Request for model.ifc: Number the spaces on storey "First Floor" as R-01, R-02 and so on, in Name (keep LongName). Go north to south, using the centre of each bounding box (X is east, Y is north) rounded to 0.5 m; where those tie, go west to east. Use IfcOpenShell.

First a look at what the model holds.

```python
import ifcopenshell
import ifcopenshell.util.element
import ifcopenshell.util.placement

model = ifcopenshell.open("model.ifc")
print(model.schema)
storey = next(s for s in model.by_type("IfcBuildingStorey") if s.Name == "First Floor")
spaces = [e for e in ifcopenshell.util.element.get_decomposition(storey) if e.is_a("IfcSpace")]
for e in sorted(spaces, key=lambda e: e.id()):
    origin = ifcopenshell.util.placement.get_local_placement(e.ObjectPlacement)[:3, 3]
    print(e.id(), e.Name, e.LongName, origin.round(2) + 0.0, sep=" | ")
```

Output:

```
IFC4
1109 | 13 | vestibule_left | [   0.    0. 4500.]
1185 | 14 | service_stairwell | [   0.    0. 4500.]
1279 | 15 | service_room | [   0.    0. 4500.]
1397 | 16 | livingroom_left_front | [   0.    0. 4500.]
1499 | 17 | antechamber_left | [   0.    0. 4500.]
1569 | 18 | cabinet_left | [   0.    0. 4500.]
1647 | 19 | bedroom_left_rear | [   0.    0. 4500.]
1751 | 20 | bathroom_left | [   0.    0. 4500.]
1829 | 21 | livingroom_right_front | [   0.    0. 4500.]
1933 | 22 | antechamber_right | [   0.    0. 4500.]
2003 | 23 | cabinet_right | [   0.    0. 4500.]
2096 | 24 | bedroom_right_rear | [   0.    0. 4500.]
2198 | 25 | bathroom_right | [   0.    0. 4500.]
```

```python
import ifcopenshell
import ifcopenshell.geom
import ifcopenshell.util.element
import ifcopenshell.util.shape

model = ifcopenshell.open("model.ifc")
settings = ifcopenshell.geom.settings()
settings.set("use-world-coords", True)


def centre(element):
    shape = ifcopenshell.geom.create_shape(settings, element)
    return ifcopenshell.util.shape.get_bbox_centroid(shape.geometry)


storey = next(s for s in model.by_type("IfcBuildingStorey") if s.Name == "First Floor")
spaces = [e for e in ifcopenshell.util.element.get_decomposition(storey) if e.is_a("IfcSpace")]

# Insertion points can sit at a corner or the storey origin, so sort by the geometry (in metres).
centres = {e: centre(e) for e in spaces}
spaces.sort(key=lambda e: (-round(centres[e][1] / 0.5), centres[e][0]))

for i, e in enumerate(spaces, start=1):
    number = f"R-{i:02d}"
    e.Name = number
    print(e.id(), number)

model.write("model_v2.ifc")
```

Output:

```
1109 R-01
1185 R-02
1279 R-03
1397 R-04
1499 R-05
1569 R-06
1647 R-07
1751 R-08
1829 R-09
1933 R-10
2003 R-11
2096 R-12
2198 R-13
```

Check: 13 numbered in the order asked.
